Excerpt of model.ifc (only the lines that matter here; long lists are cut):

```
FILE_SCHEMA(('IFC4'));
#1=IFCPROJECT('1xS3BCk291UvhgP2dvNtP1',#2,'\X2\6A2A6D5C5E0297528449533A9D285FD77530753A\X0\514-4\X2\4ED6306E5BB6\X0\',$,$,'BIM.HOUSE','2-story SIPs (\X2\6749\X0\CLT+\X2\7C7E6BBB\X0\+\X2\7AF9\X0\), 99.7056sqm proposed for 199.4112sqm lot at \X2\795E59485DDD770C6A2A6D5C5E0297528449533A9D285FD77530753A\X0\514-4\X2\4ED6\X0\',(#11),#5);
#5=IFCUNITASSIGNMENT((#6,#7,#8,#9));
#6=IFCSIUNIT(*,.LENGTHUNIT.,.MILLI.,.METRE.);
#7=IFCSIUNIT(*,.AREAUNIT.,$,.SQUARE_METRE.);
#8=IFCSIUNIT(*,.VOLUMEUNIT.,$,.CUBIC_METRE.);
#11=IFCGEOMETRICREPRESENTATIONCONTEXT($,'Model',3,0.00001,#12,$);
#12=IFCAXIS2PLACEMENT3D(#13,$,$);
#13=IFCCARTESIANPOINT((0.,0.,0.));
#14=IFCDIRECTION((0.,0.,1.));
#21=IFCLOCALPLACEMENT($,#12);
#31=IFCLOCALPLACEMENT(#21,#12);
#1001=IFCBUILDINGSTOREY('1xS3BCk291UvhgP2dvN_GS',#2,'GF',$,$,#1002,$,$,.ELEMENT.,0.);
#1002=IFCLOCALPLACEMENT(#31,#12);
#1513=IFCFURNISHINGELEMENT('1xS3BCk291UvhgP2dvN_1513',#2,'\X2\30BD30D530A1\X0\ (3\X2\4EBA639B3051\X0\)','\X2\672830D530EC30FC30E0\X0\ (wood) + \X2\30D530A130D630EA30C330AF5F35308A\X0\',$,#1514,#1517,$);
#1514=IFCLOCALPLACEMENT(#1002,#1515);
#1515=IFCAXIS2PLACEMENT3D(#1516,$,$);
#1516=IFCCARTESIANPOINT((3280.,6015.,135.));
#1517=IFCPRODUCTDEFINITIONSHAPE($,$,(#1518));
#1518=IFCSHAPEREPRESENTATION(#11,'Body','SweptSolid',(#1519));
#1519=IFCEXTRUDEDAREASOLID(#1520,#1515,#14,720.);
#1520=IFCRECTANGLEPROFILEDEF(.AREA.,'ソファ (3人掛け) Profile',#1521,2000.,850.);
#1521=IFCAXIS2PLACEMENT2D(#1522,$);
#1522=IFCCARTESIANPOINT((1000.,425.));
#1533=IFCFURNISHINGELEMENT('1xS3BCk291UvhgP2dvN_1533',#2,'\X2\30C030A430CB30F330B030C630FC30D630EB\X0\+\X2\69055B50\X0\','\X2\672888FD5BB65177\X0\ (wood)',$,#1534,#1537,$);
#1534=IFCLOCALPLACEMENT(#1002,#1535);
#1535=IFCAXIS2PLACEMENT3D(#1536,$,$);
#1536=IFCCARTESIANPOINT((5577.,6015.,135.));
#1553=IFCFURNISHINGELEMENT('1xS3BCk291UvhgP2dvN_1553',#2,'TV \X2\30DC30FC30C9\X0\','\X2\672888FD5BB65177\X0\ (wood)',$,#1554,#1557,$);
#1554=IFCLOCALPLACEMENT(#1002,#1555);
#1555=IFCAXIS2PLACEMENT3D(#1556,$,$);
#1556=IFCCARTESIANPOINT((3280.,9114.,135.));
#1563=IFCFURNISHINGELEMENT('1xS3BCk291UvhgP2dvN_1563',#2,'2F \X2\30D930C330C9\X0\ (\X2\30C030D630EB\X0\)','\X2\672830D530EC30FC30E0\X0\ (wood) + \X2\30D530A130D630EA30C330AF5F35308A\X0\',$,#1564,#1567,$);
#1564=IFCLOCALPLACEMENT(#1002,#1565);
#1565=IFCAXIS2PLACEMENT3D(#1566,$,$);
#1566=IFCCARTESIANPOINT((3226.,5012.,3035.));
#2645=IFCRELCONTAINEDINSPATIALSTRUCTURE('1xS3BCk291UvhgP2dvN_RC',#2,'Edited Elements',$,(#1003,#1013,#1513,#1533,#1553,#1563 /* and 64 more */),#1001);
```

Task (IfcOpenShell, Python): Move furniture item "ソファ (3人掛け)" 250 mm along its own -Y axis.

```python
import ifcopenshell
import ifcopenshell.api.geometry
import ifcopenshell.util.placement
import ifcopenshell.util.unit

model = ifcopenshell.open("model.ifc")
unit_scale = ifcopenshell.util.unit.calculate_unit_scale(model)

item = model.by_id(1513)
matrix = ifcopenshell.util.placement.get_local_placement(item.ObjectPlacement)
matrix[:3, 3] -= matrix[:3, 1] * 0.25 / unit_scale
ifcopenshell.api.geometry.edit_object_placement(model, product=item, matrix=matrix, is_si=False)

print(ifcopenshell.util.placement.get_local_placement(item.ObjectPlacement).round(3) + 0.0)

model.write("model-out.ifc")
```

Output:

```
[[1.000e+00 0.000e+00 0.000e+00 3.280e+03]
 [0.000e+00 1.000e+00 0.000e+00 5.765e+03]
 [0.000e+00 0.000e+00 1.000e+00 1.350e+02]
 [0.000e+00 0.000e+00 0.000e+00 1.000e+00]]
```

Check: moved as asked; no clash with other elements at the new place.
